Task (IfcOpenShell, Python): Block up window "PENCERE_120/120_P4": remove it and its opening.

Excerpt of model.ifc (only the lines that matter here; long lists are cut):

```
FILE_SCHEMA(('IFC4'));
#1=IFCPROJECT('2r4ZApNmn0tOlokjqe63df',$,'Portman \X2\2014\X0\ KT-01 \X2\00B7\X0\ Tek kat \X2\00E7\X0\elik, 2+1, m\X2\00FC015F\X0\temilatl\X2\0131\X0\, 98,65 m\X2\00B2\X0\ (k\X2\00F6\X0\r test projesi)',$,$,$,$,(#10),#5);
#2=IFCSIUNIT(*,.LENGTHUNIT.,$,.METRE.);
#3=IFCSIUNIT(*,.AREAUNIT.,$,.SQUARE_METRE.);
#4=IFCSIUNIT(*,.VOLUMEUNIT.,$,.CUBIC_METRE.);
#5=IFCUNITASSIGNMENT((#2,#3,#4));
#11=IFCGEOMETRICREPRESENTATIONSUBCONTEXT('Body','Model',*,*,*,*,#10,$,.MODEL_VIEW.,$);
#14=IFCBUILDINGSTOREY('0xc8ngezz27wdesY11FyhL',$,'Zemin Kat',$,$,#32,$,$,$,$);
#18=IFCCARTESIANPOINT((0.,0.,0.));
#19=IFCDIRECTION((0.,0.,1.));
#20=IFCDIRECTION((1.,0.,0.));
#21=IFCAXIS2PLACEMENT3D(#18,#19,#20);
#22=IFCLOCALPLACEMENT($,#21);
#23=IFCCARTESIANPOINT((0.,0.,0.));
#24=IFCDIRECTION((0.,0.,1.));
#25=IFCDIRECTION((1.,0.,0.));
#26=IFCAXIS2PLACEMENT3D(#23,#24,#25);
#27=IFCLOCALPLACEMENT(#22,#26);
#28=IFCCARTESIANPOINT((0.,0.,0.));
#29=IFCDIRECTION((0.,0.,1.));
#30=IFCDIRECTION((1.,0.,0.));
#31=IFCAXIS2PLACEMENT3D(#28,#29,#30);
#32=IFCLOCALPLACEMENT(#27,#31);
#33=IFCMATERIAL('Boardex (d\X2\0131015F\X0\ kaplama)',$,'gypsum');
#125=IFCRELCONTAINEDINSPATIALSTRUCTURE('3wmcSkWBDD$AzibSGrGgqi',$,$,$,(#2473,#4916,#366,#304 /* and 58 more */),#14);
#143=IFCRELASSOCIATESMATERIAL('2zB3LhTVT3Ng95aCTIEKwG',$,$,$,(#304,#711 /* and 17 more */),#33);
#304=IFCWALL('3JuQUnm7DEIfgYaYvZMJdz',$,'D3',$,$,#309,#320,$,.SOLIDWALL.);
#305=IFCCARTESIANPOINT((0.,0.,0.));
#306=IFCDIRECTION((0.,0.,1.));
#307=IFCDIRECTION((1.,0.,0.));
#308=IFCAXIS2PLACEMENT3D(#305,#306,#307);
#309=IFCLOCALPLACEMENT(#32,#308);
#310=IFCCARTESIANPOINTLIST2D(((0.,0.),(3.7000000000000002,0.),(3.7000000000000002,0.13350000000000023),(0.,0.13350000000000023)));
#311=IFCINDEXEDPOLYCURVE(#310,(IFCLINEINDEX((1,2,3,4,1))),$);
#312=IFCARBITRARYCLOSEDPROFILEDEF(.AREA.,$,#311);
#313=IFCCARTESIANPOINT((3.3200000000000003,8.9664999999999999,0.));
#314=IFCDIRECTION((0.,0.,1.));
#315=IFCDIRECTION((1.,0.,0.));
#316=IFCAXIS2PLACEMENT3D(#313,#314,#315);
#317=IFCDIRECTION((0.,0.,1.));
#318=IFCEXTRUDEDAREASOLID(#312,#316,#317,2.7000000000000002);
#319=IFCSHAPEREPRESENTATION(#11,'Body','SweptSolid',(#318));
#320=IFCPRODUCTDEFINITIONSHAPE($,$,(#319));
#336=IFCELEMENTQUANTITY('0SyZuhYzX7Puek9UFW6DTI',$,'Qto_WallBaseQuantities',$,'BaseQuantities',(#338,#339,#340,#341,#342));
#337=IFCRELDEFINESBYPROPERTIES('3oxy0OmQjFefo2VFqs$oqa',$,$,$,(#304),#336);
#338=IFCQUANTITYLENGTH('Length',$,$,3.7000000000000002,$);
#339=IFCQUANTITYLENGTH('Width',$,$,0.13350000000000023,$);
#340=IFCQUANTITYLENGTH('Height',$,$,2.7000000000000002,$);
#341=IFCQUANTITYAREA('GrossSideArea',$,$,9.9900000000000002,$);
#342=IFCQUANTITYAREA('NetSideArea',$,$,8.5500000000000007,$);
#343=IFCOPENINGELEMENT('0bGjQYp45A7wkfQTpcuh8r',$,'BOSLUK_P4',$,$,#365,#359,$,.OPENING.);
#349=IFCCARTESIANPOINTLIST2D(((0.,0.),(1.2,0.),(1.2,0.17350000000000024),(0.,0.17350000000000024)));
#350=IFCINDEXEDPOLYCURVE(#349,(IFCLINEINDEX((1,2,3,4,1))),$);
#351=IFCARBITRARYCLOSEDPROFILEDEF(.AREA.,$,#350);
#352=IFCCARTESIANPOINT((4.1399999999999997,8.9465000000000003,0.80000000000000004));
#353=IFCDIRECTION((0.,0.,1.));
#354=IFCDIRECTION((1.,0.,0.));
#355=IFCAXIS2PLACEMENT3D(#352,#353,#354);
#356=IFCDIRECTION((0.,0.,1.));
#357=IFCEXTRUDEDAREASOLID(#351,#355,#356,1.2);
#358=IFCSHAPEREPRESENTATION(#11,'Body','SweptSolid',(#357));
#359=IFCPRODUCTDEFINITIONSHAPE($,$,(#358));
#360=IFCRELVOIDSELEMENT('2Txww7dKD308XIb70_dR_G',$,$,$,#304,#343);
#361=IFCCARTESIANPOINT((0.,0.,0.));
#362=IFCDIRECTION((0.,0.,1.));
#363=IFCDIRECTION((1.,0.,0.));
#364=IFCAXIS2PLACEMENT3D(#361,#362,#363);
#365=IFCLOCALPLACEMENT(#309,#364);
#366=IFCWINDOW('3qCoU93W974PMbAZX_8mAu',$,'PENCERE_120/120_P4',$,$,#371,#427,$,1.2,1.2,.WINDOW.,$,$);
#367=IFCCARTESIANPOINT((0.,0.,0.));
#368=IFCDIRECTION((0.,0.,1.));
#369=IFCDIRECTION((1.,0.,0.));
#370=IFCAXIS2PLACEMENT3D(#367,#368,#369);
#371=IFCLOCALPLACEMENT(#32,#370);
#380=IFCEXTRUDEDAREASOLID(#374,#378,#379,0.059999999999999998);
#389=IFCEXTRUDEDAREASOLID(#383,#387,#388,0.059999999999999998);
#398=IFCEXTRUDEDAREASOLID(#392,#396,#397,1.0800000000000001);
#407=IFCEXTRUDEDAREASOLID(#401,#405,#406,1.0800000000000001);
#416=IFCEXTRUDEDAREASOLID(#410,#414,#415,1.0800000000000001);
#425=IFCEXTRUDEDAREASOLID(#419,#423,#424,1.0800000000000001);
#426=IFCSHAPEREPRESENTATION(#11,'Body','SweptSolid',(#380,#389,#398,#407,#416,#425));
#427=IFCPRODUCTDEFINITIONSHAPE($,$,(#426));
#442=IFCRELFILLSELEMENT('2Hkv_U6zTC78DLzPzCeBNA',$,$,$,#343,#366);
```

```python
import ifcopenshell
import ifcopenshell.api.feature
import ifcopenshell.api.pset
import ifcopenshell.api.root
import ifcopenshell.geom
import ifcopenshell.util.element
import ifcopenshell.util.shape
import ifcopenshell.util.unit

model = ifcopenshell.open("model.ifc")
area_scale = ifcopenshell.util.unit.calculate_unit_scale(model, "AREAUNIT")
settings = ifcopenshell.geom.settings()


def volume(element):
    """Net volume in cubic metres, openings subtracted."""
    shape = ifcopenshell.geom.create_shape(settings, element)
    return ifcopenshell.util.shape.get_volume(shape.geometry)


window = model.by_id(366)
opening = window.FillsVoids[0].RelatingOpeningElement
wall = opening.VoidsElements[0].RelatingBuildingElement
before = volume(wall)

ifcopenshell.api.root.remove_product(model, product=window)
ifcopenshell.api.feature.remove_feature(model, feature=opening)

after = volume(wall)
thickness = 0.1335  # wall thickness in metres

# Update the wall's stored quantities.
qto = model.by_id(ifcopenshell.util.element.get_pset(wall, "Qto_WallBaseQuantities", should_inherit=False)["id"])
ifcopenshell.api.pset.edit_qto(model, qto=qto, properties={"NetSideArea": after / thickness / area_scale})

print(f"wall volume {before:.3f} -> {after:.3f} m3")

model.write("model-out.ifc")
```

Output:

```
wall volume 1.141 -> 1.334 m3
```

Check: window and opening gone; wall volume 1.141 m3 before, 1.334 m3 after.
